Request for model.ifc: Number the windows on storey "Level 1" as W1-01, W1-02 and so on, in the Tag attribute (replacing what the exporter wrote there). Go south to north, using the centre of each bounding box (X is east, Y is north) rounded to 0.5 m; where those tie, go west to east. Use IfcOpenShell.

First a look at what the model holds.

```python
import ifcopenshell
import ifcopenshell.util.element
import ifcopenshell.util.placement

model = ifcopenshell.open("model.ifc")
print(model.schema)
storey = next(s for s in model.by_type("IfcBuildingStorey") if s.Name == "Level 1")
windows = [e for e in ifcopenshell.util.element.get_decomposition(storey) if e.is_a("IfcWindow")]
for e in sorted(windows, key=lambda e: e.id()):
    origin = ifcopenshell.util.placement.get_local_placement(e.ObjectPlacement)[:3, 3]
    print(e.id(), e.Tag, e.Name, origin.round(2) + 0.0, sep=" | ")
```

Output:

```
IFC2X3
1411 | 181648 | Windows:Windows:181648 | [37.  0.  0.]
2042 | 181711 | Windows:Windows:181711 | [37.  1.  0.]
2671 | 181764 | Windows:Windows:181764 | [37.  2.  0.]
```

```python
import ifcopenshell
import ifcopenshell.geom
import ifcopenshell.util.element
import ifcopenshell.util.shape

model = ifcopenshell.open("model.ifc")
settings = ifcopenshell.geom.settings()
settings.set("use-world-coords", True)


def centre(element):
    shape = ifcopenshell.geom.create_shape(settings, element)
    return ifcopenshell.util.shape.get_bbox_centroid(shape.geometry)


storey = next(s for s in model.by_type("IfcBuildingStorey") if s.Name == "Level 1")
windows = [e for e in ifcopenshell.util.element.get_decomposition(storey) if e.is_a("IfcWindow")]

# Insertion points can sit at a corner or the storey origin, so sort by the geometry (in metres).
centres = {e: centre(e) for e in windows}
windows.sort(key=lambda e: (round(centres[e][1] / 0.5), centres[e][0]))

for i, e in enumerate(windows, start=1):
    number = f"W1-{i:02d}"
    e.Tag = number
    print(e.id(), number)

model.write("model_updated.ifc")
```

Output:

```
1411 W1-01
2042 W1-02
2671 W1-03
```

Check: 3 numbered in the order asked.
